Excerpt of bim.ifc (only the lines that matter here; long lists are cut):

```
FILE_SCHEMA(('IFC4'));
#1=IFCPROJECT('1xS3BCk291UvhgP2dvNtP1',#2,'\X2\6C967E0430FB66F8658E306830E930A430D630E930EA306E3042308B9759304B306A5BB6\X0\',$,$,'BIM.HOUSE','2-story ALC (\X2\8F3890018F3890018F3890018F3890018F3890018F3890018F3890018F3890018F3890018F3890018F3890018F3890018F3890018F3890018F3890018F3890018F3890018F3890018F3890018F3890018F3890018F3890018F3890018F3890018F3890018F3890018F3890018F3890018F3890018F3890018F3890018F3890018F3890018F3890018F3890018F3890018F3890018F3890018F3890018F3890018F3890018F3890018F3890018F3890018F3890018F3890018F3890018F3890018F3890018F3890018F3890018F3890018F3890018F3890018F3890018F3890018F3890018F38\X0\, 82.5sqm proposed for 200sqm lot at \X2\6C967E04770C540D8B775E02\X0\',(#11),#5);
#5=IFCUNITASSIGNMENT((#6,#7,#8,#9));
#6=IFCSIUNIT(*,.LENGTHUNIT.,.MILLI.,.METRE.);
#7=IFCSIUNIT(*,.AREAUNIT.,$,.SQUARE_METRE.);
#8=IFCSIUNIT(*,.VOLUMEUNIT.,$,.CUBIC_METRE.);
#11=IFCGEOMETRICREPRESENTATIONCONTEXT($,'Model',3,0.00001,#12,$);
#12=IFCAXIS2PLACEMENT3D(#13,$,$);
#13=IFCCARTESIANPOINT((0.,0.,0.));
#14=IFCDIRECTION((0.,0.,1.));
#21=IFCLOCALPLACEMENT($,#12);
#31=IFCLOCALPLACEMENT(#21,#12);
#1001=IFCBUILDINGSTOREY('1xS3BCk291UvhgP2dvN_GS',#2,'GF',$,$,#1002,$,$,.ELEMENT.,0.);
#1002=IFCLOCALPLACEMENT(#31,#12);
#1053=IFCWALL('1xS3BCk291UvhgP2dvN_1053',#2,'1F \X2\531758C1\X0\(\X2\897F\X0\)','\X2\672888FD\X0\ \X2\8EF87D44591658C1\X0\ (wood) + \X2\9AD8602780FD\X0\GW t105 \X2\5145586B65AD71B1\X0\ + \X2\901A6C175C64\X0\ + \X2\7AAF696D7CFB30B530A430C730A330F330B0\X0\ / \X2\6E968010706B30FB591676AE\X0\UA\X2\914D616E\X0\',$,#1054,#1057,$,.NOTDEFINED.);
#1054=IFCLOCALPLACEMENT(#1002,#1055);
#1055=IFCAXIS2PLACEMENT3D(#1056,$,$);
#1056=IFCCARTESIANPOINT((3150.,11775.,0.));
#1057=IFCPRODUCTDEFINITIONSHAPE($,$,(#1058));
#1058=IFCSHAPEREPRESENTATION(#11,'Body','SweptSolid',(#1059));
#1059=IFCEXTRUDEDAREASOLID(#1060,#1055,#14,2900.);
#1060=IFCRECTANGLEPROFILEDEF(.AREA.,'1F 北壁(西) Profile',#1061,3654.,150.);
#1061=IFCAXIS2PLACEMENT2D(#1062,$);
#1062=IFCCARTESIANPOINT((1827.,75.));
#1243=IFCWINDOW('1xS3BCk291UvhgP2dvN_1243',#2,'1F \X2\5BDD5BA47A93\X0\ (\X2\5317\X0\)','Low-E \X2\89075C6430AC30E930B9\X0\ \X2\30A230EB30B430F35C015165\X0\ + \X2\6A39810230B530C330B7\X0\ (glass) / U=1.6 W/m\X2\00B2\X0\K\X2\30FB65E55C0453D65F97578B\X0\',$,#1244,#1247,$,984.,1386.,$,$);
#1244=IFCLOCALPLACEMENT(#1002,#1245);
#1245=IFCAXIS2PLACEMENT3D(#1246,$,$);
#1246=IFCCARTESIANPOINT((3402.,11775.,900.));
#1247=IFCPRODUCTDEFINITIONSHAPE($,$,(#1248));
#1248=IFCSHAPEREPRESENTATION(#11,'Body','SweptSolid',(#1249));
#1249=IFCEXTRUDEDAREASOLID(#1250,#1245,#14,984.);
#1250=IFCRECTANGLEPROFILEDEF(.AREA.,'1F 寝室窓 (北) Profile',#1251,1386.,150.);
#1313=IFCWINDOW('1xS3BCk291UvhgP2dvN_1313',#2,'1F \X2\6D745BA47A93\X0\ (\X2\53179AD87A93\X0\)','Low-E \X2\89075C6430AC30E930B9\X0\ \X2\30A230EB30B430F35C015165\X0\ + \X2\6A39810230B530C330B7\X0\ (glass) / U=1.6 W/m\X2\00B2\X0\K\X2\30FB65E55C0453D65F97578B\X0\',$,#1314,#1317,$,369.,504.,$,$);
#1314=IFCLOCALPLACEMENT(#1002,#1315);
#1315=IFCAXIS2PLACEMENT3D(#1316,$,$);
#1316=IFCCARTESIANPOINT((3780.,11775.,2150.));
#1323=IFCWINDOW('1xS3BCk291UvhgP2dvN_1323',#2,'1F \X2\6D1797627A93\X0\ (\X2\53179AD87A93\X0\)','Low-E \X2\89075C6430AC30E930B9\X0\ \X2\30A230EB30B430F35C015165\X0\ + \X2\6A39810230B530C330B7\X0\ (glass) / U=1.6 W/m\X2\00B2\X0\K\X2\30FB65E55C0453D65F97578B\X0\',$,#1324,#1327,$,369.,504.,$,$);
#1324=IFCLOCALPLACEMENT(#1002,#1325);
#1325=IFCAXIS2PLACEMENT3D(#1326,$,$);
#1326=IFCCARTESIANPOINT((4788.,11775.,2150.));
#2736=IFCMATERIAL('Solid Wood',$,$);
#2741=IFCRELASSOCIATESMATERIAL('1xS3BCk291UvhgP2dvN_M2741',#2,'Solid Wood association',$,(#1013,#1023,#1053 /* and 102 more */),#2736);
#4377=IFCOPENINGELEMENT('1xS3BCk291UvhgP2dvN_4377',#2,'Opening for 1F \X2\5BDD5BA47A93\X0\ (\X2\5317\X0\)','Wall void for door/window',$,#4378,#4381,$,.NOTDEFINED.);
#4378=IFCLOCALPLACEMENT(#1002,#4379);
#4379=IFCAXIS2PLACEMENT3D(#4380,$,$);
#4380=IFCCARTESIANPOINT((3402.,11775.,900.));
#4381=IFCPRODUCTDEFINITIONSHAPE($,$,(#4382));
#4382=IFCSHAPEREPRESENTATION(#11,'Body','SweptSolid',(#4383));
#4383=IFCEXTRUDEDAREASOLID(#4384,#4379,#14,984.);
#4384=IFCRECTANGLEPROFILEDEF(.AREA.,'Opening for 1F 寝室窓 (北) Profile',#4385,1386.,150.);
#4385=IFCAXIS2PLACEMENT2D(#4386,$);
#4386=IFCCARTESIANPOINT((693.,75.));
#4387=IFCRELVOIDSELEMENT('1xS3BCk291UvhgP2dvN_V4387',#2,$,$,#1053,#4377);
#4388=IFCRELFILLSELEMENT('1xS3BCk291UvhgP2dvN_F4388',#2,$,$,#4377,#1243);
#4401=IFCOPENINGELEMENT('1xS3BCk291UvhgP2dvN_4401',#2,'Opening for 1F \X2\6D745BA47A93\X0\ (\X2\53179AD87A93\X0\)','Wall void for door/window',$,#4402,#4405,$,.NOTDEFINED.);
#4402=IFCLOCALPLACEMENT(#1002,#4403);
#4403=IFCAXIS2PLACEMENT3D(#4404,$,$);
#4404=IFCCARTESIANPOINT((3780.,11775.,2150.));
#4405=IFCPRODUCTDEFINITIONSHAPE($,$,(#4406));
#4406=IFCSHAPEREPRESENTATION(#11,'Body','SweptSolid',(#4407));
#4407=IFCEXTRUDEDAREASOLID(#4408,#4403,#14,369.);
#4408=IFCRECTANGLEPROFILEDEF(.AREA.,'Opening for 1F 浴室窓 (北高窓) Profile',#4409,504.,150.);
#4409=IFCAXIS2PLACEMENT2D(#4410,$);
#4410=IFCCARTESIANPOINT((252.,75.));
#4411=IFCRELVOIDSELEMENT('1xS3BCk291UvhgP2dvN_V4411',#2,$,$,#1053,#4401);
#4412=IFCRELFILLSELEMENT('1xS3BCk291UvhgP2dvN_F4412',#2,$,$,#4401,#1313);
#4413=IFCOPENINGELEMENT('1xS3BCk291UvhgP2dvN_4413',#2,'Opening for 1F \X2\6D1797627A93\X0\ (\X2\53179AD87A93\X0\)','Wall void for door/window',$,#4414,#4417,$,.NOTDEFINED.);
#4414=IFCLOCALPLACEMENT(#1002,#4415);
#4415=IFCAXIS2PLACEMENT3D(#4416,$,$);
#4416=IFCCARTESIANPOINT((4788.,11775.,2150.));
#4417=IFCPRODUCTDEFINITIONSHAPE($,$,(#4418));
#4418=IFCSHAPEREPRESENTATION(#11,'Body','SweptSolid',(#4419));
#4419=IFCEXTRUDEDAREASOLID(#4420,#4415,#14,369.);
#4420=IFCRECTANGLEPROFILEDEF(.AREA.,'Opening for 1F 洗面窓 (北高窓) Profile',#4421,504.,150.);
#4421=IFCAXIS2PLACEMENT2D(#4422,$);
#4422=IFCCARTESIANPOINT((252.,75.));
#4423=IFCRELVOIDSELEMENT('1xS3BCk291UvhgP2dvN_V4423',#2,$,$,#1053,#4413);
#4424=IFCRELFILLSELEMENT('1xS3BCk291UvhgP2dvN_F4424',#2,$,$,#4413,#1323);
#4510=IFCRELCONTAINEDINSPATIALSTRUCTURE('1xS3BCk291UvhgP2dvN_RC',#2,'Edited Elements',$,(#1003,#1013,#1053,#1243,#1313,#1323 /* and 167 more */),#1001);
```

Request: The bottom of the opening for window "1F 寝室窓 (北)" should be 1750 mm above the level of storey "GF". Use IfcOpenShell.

```python
import numpy as np
import ifcopenshell
import ifcopenshell.api.geometry
import ifcopenshell.geom
import ifcopenshell.util.element
import ifcopenshell.util.placement
import ifcopenshell.util.shape
import ifcopenshell.util.unit

model = ifcopenshell.open("bim.ifc")
unit_scale = ifcopenshell.util.unit.calculate_unit_scale(model)

window = model.by_guid("1xS3BCk291UvhgP2dvN_1243")
opening = window.FillsVoids[0].RelatingOpeningElement
storey = ifcopenshell.util.element.get_container(window, ifc_class="IfcBuildingStorey")
level = ifcopenshell.util.placement.get_local_placement(storey.ObjectPlacement)[2, 3]

# The opening's origin need not be at the sill, so measure its lowest point.
shape = ifcopenshell.geom.create_shape(ifcopenshell.geom.settings(), opening)
bottom = ifcopenshell.util.shape.get_shape_bottom_elevation(shape, shape.geometry) / unit_scale
dz = level + 1750.0 - bottom

shift = np.array([0.0, 0.0, dz])
# The window is not placed relative to its opening, so move both.
for product in (opening, window):
    matrix = ifcopenshell.util.placement.get_local_placement(product.ObjectPlacement)
    matrix[:3, 3] += shift
    ifcopenshell.api.geometry.edit_object_placement(model, product=product, matrix=matrix, is_si=False)

print(f"moved by {dz * unit_scale:+.3f} m")

model.write("bim_updated.ifc")
```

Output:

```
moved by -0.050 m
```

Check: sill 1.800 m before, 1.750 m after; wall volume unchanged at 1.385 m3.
